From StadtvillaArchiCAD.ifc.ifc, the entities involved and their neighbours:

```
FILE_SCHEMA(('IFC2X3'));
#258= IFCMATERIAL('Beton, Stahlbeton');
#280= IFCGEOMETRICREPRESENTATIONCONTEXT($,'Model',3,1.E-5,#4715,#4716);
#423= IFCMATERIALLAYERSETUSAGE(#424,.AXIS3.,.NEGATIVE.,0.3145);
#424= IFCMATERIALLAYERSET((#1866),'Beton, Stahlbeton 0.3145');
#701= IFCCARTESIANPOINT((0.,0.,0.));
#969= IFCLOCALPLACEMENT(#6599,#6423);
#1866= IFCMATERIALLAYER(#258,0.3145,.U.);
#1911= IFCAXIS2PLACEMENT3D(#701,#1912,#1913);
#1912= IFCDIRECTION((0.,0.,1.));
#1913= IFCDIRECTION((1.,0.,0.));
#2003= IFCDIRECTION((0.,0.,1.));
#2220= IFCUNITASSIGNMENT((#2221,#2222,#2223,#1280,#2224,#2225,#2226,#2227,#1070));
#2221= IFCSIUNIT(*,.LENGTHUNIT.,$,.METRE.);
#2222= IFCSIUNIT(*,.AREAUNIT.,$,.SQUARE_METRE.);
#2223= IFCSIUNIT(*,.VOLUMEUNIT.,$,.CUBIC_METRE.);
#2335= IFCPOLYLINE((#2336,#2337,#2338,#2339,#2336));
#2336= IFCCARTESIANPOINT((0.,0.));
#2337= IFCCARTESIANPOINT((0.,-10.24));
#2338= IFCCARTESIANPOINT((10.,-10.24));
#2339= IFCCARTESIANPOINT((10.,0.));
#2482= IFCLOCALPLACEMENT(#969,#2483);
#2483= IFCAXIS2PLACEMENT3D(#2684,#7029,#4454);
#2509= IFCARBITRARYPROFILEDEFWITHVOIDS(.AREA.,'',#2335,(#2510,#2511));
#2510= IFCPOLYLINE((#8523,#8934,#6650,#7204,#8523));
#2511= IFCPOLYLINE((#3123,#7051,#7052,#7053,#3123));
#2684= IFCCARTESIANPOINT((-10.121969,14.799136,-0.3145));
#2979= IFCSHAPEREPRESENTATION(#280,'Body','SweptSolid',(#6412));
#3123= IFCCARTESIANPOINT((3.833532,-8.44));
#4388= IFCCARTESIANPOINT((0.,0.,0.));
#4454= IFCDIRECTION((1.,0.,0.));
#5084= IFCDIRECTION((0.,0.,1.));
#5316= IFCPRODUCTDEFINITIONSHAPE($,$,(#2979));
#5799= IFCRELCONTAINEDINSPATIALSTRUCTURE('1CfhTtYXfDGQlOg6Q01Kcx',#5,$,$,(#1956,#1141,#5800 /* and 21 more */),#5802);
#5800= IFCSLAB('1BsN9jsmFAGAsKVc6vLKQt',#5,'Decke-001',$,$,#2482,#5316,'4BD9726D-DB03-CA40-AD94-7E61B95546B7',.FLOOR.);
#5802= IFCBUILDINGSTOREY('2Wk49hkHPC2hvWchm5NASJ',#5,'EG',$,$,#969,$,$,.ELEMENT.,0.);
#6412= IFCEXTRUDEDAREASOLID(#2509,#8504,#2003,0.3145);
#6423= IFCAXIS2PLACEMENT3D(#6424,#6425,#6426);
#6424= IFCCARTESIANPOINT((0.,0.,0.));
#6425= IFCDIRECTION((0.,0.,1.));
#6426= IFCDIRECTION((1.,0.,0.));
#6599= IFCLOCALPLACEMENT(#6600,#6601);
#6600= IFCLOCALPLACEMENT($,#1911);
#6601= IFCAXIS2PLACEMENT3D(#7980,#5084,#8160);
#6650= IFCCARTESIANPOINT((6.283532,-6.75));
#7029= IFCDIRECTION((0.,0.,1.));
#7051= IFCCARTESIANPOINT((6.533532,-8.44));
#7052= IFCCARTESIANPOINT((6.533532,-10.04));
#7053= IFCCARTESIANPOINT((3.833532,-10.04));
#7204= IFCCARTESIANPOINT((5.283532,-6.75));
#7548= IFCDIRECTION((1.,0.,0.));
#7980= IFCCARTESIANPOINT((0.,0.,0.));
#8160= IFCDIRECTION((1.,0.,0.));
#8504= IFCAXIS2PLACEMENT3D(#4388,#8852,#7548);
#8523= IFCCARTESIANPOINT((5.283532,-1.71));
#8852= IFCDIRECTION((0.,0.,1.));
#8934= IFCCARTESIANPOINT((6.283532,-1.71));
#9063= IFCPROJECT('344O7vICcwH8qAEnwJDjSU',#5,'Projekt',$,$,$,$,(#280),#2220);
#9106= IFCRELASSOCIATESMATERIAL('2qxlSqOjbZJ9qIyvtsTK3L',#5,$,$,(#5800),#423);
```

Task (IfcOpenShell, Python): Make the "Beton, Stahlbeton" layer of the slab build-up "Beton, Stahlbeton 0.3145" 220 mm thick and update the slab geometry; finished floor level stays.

```python
import ifcopenshell
import ifcopenshell.util.element
import ifcopenshell.util.unit

model = ifcopenshell.open("StadtvillaArchiCAD.ifc.ifc")
unit_scale = ifcopenshell.util.unit.calculate_unit_scale(model)

layer_set = model.by_id(424)
layer = next(l for l in layer_set.MaterialLayers if l.Material and l.Material.Name == "Beton, Stahlbeton")
change = 0.22 / unit_scale - layer.LayerThickness
layer.LayerThickness += change

# Geometry does not follow the layer set by itself.
slabs = [e for e in ifcopenshell.util.element.get_elements_by_material(model, layer_set) if e.is_a("IfcSlab")]
for slab in sorted(slabs, key=lambda e: e.id()):
    body = next(r for r in slab.Representation.Representations if r.RepresentationIdentifier == "Body")
    solid = body.Items[0]
    old_depth = solid.Depth
    solid.Depth += change
    # Extruded upwards: lower the start of the extrusion so the top stays.
    x, y, z = solid.Position.Location.Coordinates
    solid.Position.Location = model.createIfcCartesianPoint((x, y, z - change))
    print(slab.id(), f"{old_depth:g} -> {solid.Depth:g}")

model.write("StadtvillaArchiCAD.ifc_v2.ifc")
```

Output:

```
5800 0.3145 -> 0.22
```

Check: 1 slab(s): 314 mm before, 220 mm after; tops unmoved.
